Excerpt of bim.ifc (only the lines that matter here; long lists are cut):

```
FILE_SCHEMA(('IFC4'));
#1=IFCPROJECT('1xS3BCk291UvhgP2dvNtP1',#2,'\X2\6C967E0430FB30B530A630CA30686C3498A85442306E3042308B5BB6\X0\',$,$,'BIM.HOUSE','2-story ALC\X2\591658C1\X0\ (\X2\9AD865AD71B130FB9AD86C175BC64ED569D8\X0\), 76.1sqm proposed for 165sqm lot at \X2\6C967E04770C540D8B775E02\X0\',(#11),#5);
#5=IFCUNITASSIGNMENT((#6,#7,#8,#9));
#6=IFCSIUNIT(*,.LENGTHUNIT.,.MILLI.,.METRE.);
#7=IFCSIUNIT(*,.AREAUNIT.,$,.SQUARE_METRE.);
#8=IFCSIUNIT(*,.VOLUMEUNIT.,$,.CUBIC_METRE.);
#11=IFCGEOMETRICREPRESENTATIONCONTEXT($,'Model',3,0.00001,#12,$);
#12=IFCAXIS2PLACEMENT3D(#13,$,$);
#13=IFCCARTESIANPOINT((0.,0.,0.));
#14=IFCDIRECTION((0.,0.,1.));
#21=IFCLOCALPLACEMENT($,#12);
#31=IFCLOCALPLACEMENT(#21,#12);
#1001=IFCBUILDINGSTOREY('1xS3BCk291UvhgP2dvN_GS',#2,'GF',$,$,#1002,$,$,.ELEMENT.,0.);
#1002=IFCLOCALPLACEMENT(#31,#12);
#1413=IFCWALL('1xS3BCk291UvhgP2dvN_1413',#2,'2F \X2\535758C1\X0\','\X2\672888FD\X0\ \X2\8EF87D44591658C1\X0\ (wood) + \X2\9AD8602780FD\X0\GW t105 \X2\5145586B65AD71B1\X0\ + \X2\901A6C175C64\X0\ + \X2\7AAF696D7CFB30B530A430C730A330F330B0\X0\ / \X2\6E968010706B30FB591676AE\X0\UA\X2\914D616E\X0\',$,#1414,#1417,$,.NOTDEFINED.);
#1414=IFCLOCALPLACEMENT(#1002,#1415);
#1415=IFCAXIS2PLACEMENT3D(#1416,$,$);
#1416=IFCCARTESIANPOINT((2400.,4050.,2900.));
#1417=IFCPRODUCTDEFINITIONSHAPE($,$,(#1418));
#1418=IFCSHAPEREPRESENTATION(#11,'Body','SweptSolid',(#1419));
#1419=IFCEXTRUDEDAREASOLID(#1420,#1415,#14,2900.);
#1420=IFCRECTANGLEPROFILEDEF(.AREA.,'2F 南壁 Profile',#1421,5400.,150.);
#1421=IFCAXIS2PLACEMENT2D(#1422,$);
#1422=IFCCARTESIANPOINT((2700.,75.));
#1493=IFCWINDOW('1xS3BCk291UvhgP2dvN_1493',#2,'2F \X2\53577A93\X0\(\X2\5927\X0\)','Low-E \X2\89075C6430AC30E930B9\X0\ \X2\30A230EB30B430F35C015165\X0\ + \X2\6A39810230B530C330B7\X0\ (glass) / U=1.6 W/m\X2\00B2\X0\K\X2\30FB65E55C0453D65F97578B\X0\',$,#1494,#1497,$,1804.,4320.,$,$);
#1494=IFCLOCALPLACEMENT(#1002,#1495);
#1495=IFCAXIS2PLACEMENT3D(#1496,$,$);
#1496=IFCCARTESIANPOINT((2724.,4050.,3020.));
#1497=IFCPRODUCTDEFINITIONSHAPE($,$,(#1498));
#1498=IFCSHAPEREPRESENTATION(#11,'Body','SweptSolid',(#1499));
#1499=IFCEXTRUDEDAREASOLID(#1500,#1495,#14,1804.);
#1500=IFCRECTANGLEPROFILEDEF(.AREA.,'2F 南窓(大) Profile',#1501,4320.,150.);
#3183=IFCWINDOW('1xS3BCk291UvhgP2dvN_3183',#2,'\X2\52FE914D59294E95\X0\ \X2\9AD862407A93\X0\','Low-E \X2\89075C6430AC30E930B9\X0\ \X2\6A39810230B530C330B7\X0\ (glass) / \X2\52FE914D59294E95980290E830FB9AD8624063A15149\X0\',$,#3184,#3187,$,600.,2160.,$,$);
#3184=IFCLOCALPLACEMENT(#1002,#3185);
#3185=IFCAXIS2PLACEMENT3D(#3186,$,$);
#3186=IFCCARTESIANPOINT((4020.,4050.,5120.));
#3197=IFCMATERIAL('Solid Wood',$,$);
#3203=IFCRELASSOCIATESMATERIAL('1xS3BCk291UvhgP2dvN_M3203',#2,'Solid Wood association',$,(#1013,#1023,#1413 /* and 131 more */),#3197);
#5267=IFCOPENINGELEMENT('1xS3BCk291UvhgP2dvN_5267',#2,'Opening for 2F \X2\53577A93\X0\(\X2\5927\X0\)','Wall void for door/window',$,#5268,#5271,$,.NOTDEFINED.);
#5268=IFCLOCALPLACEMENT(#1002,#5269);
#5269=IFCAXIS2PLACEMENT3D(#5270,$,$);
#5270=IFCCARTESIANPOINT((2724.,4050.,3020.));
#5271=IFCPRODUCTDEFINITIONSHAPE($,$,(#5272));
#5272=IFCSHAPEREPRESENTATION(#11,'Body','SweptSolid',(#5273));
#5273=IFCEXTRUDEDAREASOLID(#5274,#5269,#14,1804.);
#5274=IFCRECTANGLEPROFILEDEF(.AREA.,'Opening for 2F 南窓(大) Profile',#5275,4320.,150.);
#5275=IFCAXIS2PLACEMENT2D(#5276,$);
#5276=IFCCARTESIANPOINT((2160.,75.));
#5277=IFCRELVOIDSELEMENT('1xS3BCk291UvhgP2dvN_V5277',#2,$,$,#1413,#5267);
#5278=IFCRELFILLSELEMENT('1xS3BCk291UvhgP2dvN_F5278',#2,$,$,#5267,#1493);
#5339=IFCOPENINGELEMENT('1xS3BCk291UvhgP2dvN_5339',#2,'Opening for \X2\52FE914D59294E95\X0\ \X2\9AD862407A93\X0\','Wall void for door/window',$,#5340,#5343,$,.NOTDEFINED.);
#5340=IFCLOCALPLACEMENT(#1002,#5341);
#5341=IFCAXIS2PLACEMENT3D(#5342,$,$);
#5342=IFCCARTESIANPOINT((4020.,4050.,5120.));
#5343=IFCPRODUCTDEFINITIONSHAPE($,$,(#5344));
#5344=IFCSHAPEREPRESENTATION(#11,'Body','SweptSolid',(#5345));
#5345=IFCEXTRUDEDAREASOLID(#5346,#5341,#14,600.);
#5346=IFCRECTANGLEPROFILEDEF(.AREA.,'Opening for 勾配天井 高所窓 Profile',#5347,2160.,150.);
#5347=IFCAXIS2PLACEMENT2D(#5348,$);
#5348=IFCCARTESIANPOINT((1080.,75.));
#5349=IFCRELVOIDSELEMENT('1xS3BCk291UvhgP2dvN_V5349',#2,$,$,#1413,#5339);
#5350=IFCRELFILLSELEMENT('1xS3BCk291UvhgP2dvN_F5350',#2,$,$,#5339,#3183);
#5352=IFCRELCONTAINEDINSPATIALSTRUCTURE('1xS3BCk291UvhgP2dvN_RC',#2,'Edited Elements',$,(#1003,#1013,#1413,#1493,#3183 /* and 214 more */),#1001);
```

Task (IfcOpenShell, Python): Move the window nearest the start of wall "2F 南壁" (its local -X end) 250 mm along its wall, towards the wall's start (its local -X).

```python
import ifcopenshell
import ifcopenshell.api.geometry
import ifcopenshell.util.placement
import ifcopenshell.util.unit

model = ifcopenshell.open("bim.ifc")
unit_scale = ifcopenshell.util.unit.calculate_unit_scale(model)

window = model.by_id(1493)
opening = window.FillsVoids[0].RelatingOpeningElement
wall = opening.VoidsElements[0].RelatingBuildingElement

wall_matrix = ifcopenshell.util.placement.get_local_placement(wall.ObjectPlacement)
shift = wall_matrix[:3, 0] * -0.25 / unit_scale
before = ifcopenshell.util.placement.get_local_placement(window.ObjectPlacement)[:3, 3].copy()

# The window is not placed relative to its opening, so move both.
for product in (opening, window):
    matrix = ifcopenshell.util.placement.get_local_placement(product.ObjectPlacement)
    matrix[:3, 3] += shift
    ifcopenshell.api.geometry.edit_object_placement(model, product=product, matrix=matrix, is_si=False)

after = ifcopenshell.util.placement.get_local_placement(window.ObjectPlacement)[:3, 3]
print("window moved by", (after - before).round(3) + 0.0)

model.write("bim_updated.ifc")
```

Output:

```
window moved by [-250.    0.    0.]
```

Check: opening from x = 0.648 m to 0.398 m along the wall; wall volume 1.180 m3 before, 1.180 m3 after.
